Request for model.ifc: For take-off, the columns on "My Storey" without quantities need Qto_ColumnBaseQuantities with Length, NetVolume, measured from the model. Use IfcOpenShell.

First a look at what the model holds.

```python
import ifcopenshell
import ifcopenshell.util.element
import ifcopenshell.util.unit

model = ifcopenshell.open("model.ifc")
print(model.schema)
for unit_type in ("LENGTHUNIT", "AREAUNIT", "VOLUMEUNIT"):
    print(unit_type, ifcopenshell.util.unit.calculate_unit_scale(model, unit_type))
storey = next(s for s in model.by_type("IfcBuildingStorey") if s.Name == "My Storey")
columns = [e for e in ifcopenshell.util.element.get_decomposition(storey) if e.is_a("IfcColumn")]
for e in sorted(columns, key=lambda e: e.id()):
    print(e.id(), e.is_a(), e.Name, list(ifcopenshell.util.element.get_psets(e, qtos_only=True)), sep=" | ")
```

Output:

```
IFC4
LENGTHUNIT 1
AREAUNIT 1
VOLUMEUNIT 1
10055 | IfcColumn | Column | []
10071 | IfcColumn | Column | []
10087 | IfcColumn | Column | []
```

```python
import ifcopenshell
import ifcopenshell.api.pset
import ifcopenshell.geom
import ifcopenshell.util.element
import ifcopenshell.util.shape
import ifcopenshell.util.unit

model = ifcopenshell.open("model.ifc")
unit_scale = ifcopenshell.util.unit.calculate_unit_scale(model)
volume_scale = ifcopenshell.util.unit.calculate_unit_scale(model, "VOLUMEUNIT")
settings = ifcopenshell.geom.settings()

storey = next(s for s in model.by_type("IfcBuildingStorey") if s.Name == "My Storey")
columns = [e for e in ifcopenshell.util.element.get_decomposition(storey) if e.is_a("IfcColumn")]

for e in sorted(columns, key=lambda e: e.id()):
    if ifcopenshell.util.element.get_psets(e, qtos_only=True, should_inherit=False):
        continue
    # Geometry comes back in metres, in the element's own axes.
    shape = ifcopenshell.geom.create_shape(settings, e)
    values = {
        "Length": ifcopenshell.util.shape.get_z(shape.geometry) / unit_scale,
        "NetVolume": ifcopenshell.util.shape.get_volume(shape.geometry) / volume_scale,
    }
    qto = ifcopenshell.api.pset.add_qto(model, product=e, name="Qto_ColumnBaseQuantities")
    ifcopenshell.api.pset.edit_qto(model, qto=qto, properties=values)
    print(e.id(), {k: round(v, 3) for k, v in values.items()})

model.write("model_rev.ifc")
```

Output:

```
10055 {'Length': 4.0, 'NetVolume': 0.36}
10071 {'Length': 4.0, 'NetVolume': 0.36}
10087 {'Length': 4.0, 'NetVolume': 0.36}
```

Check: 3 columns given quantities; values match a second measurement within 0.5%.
